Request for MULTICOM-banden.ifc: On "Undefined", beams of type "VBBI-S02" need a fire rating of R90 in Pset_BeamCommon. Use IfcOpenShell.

First a look at what the model holds.

```python
import ifcopenshell
import ifcopenshell.util.element

model = ifcopenshell.open("MULTICOM-banden.ifc")
print(model.schema)
storey = next(s for s in model.by_type("IfcBuildingStorey") if s.Name == "Undefined")
beams = [e for e in ifcopenshell.util.element.get_decomposition(storey) if e.is_a("IfcBeam")]
seen = {}
for e in beams:
    element_type = ifcopenshell.util.element.get_type(e)
    key = (element_type.Name if element_type != e and element_type else None, ifcopenshell.util.element.get_pset(e, "Pset_BeamCommon", "FireRating"))
    seen[key] = seen.get(key, 0) + 1
for (name, value), count in sorted(seen.items(), key=str):
    print(count, "x", name, "|", value)
```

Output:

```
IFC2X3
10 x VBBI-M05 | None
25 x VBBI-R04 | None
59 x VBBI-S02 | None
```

```python
import ifcopenshell
import ifcopenshell.api.pset
import ifcopenshell.util.element

model = ifcopenshell.open("MULTICOM-banden.ifc")

storey = next(s for s in model.by_type("IfcBuildingStorey") if s.Name == "Undefined")
beams = [e for e in ifcopenshell.util.element.get_decomposition(storey) if e.is_a("IfcBeam")]

count = 0
for e in beams:
    element_type = ifcopenshell.util.element.get_type(e)
    if element_type in (None, e) or element_type.Name != "VBBI-S02":
        continue
    # add_pset returns the element's existing set when there is one.
    pset = ifcopenshell.api.pset.add_pset(model, product=e, name="Pset_BeamCommon")
    ifcopenshell.api.pset.edit_pset(model, pset=pset, properties={"FireRating": "R90"})
    count += 1

print(count, "beams updated")

model.write("MULTICOM-banden_rev.ifc")
```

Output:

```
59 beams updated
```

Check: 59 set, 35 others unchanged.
